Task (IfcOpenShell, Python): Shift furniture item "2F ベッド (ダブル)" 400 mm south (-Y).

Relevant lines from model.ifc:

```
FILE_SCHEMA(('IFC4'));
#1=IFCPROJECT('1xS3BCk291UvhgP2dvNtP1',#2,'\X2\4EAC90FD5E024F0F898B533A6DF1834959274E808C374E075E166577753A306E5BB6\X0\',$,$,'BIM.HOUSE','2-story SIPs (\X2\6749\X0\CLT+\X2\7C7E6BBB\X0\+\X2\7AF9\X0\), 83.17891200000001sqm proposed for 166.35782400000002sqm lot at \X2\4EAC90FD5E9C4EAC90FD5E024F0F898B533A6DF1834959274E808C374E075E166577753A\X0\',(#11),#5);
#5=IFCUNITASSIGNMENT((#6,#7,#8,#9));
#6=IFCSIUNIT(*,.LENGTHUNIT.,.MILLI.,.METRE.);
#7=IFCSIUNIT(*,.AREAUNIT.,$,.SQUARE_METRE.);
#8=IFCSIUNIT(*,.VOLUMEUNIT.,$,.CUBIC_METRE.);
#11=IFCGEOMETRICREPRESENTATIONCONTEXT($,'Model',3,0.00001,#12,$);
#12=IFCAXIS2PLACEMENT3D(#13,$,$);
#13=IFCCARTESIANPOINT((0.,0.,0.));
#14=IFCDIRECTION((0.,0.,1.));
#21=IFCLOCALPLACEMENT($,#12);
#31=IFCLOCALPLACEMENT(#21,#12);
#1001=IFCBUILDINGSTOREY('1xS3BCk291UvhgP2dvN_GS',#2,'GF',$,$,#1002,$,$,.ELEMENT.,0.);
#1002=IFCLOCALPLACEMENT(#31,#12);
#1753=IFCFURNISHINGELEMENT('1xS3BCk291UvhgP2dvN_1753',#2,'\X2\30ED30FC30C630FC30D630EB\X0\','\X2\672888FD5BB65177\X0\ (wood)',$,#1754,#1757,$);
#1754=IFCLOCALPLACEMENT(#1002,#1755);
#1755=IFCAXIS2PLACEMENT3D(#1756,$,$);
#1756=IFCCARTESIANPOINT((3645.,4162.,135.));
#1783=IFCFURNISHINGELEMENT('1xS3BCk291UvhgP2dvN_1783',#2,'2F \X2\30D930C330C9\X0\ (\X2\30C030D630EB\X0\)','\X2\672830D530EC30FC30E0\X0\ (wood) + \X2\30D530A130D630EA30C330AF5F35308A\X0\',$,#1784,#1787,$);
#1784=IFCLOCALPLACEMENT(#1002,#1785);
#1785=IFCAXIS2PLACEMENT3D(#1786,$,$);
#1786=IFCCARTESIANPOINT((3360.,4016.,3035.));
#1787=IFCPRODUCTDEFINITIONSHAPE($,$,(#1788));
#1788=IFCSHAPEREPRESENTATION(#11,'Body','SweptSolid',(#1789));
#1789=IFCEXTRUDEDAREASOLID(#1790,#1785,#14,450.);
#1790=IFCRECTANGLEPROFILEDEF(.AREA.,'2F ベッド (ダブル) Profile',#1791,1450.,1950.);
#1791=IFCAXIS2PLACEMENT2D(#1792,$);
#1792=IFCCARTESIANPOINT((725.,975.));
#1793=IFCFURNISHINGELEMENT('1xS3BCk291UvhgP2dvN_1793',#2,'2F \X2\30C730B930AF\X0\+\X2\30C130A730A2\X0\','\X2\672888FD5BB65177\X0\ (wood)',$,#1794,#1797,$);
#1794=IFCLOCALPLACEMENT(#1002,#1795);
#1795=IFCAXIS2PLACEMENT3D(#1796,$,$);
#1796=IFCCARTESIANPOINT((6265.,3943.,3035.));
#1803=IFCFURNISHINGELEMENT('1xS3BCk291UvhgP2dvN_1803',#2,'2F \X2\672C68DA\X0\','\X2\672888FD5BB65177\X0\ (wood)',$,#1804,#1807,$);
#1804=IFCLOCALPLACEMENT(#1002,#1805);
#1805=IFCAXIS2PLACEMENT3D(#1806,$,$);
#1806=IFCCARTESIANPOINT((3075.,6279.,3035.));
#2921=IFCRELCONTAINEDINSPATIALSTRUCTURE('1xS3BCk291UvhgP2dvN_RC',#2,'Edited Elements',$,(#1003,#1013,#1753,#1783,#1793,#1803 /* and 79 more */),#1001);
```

```python
import ifcopenshell
import ifcopenshell.api.geometry
import ifcopenshell.util.placement

model = ifcopenshell.open("model.ifc")

item = model.by_id(1783)
matrix = ifcopenshell.util.placement.get_local_placement(item.ObjectPlacement)
matrix[1, 3] -= 400.0
ifcopenshell.api.geometry.edit_object_placement(model, product=item, matrix=matrix, is_si=False)

print(ifcopenshell.util.placement.get_local_placement(item.ObjectPlacement).round(3) + 0.0)

model.write("model_rev.ifc")
```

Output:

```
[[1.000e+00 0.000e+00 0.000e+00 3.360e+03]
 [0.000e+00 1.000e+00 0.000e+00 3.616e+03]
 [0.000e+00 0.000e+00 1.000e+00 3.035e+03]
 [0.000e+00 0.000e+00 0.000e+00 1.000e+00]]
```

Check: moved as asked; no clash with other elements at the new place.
